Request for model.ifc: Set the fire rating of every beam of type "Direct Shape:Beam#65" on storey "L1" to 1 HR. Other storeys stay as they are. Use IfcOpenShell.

First a look at what the model holds.

```python
import ifcopenshell
import ifcopenshell.util.element

model = ifcopenshell.open("model.ifc")
print(model.schema)
storey = next(s for s in model.by_type("IfcBuildingStorey") if s.Name == "L1")
beams = [e for e in ifcopenshell.util.element.get_decomposition(storey) if e.is_a("IfcBeam")]
seen = {}
for e in beams:
    element_type = ifcopenshell.util.element.get_type(e)
    key = (element_type.Name if element_type != e and element_type else None, ifcopenshell.util.element.get_pset(e, "Pset_BeamCommon", "FireRating"))
    seen[key] = seen.get(key, 0) + 1
for (name, value), count in sorted(seen.items(), key=str):
    print(count, "x", name, "|", value)
```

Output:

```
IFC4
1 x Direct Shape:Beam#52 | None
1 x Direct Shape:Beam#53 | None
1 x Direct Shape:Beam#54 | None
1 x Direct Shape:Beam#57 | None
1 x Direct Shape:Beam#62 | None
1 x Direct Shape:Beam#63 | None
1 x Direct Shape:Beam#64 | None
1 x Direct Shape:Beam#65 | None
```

```python
import ifcopenshell
import ifcopenshell.api.pset
import ifcopenshell.util.element

model = ifcopenshell.open("model.ifc")

storey = next(s for s in model.by_type("IfcBuildingStorey") if s.Name == "L1")
beams = [e for e in ifcopenshell.util.element.get_decomposition(storey) if e.is_a("IfcBeam")]

count = 0
for e in beams:
    element_type = ifcopenshell.util.element.get_type(e)
    if element_type in (None, e) or element_type.Name != "Direct Shape:Beam#65":
        continue
    # add_pset returns the element's existing set when there is one.
    pset = ifcopenshell.api.pset.add_pset(model, product=e, name="Pset_BeamCommon")
    ifcopenshell.api.pset.edit_pset(model, pset=pset, properties={"FireRating": "1 HR"})
    count += 1

print(count, "beams updated")

model.write("model_updated.ifc")
```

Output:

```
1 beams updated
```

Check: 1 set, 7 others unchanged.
